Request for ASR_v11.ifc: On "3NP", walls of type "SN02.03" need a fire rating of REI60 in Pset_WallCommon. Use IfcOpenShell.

First a look at what the model holds.

```python
import ifcopenshell
import ifcopenshell.util.element

model = ifcopenshell.open("ASR_v11.ifc")
print(model.schema)
storey = next(s for s in model.by_type("IfcBuildingStorey") if s.Name == "3NP")
walls = [e for e in ifcopenshell.util.element.get_decomposition(storey) if e.is_a("IfcWall")]
seen = {}
for e in walls:
    element_type = ifcopenshell.util.element.get_type(e)
    key = (element_type.Name if element_type != e and element_type else None, ifcopenshell.util.element.get_pset(e, "Pset_WallCommon", "FireRating"))
    seen[key] = seen.get(key, 0) + 1
for (name, value), count in sorted(seen.items(), key=str):
    print(count, "x", name, "|", value)
```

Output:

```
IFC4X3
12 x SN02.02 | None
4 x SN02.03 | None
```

```python
import ifcopenshell
import ifcopenshell.api.pset
import ifcopenshell.util.element

model = ifcopenshell.open("ASR_v11.ifc")

storey = next(s for s in model.by_type("IfcBuildingStorey") if s.Name == "3NP")
walls = [e for e in ifcopenshell.util.element.get_decomposition(storey) if e.is_a("IfcWall")]

count = 0
for e in walls:
    element_type = ifcopenshell.util.element.get_type(e)
    if element_type in (None, e) or element_type.Name != "SN02.03":
        continue
    # add_pset returns the element's existing set when there is one.
    pset = ifcopenshell.api.pset.add_pset(model, product=e, name="Pset_WallCommon")
    ifcopenshell.api.pset.edit_pset(model, pset=pset, properties={"FireRating": "REI60"})
    count += 1

print(count, "walls updated")

model.write("ASR_v11_updated.ifc")
```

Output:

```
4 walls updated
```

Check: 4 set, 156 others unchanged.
